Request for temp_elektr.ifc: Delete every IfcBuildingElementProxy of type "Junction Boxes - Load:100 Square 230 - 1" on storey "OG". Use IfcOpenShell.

First a look at what the model holds.

```python
import ifcopenshell
import ifcopenshell.util.element

model = ifcopenshell.open("temp_elektr.ifc")
print(model.schema)
storey = next(s for s in model.by_type("IfcBuildingStorey") if s.Name == "OG")
proxies = [e for e in ifcopenshell.util.element.get_decomposition(storey) if e.is_a("IfcBuildingElementProxy")]
seen = {}
for e in proxies:
    element_type = ifcopenshell.util.element.get_type(e)
    name = element_type.Name if element_type not in (None, e) else None
    seen[name] = seen.get(name, 0) + 1
for name, count in sorted(seen.items(), key=str):
    print(count, "x", name)
```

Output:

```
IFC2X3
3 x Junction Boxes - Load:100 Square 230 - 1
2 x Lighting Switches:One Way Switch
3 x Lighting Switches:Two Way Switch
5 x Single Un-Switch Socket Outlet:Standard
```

```python
import ifcopenshell
import ifcopenshell.api.root
import ifcopenshell.util.element

model = ifcopenshell.open("temp_elektr.ifc")

storey = next(s for s in model.by_type("IfcBuildingStorey") if s.Name == "OG")
proxies = [e for e in ifcopenshell.util.element.get_decomposition(storey) if e.is_a("IfcBuildingElementProxy")]
targets = [e for e in proxies if (t := ifcopenshell.util.element.get_type(e)) not in (None, e) and t.Name == "Junction Boxes - Load:100 Square 230 - 1"]

for e in targets:
    ifcopenshell.api.root.remove_product(model, product=e)
print(len(targets), "removed")

model.write("temp_elektr_updated.ifc")
```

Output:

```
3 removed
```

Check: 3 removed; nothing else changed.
